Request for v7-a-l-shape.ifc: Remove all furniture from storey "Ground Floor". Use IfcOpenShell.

First a look at what the model holds.

```python
import ifcopenshell
import ifcopenshell.util.element

model = ifcopenshell.open("v7-a-l-shape.ifc")
print(model.schema)
storey = next(s for s in model.by_type("IfcBuildingStorey") if s.Name == "Ground Floor")
furniture = [e for e in ifcopenshell.util.element.get_decomposition(storey) if e.is_a("IfcFurnishingElement")]
seen = {}
for e in furniture:
    element_type = ifcopenshell.util.element.get_type(e)
    name = element_type.Name if element_type not in (None, e) else None
    seen[name] = seen.get(name, 0) + 1
for name, count in sorted(seen.items(), key=str):
    print(count, "x", name)
```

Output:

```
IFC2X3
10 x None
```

```python
import ifcopenshell
import ifcopenshell.api.root
import ifcopenshell.util.element

model = ifcopenshell.open("v7-a-l-shape.ifc")

storey = next(s for s in model.by_type("IfcBuildingStorey") if s.Name == "Ground Floor")
furniture = [e for e in ifcopenshell.util.element.get_decomposition(storey) if e.is_a("IfcFurnishingElement")]

for e in furniture:
    ifcopenshell.api.root.remove_product(model, product=e)
print(len(furniture), "removed")

model.write("v7-a-l-shape_updated.ifc")
```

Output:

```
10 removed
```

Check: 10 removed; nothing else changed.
